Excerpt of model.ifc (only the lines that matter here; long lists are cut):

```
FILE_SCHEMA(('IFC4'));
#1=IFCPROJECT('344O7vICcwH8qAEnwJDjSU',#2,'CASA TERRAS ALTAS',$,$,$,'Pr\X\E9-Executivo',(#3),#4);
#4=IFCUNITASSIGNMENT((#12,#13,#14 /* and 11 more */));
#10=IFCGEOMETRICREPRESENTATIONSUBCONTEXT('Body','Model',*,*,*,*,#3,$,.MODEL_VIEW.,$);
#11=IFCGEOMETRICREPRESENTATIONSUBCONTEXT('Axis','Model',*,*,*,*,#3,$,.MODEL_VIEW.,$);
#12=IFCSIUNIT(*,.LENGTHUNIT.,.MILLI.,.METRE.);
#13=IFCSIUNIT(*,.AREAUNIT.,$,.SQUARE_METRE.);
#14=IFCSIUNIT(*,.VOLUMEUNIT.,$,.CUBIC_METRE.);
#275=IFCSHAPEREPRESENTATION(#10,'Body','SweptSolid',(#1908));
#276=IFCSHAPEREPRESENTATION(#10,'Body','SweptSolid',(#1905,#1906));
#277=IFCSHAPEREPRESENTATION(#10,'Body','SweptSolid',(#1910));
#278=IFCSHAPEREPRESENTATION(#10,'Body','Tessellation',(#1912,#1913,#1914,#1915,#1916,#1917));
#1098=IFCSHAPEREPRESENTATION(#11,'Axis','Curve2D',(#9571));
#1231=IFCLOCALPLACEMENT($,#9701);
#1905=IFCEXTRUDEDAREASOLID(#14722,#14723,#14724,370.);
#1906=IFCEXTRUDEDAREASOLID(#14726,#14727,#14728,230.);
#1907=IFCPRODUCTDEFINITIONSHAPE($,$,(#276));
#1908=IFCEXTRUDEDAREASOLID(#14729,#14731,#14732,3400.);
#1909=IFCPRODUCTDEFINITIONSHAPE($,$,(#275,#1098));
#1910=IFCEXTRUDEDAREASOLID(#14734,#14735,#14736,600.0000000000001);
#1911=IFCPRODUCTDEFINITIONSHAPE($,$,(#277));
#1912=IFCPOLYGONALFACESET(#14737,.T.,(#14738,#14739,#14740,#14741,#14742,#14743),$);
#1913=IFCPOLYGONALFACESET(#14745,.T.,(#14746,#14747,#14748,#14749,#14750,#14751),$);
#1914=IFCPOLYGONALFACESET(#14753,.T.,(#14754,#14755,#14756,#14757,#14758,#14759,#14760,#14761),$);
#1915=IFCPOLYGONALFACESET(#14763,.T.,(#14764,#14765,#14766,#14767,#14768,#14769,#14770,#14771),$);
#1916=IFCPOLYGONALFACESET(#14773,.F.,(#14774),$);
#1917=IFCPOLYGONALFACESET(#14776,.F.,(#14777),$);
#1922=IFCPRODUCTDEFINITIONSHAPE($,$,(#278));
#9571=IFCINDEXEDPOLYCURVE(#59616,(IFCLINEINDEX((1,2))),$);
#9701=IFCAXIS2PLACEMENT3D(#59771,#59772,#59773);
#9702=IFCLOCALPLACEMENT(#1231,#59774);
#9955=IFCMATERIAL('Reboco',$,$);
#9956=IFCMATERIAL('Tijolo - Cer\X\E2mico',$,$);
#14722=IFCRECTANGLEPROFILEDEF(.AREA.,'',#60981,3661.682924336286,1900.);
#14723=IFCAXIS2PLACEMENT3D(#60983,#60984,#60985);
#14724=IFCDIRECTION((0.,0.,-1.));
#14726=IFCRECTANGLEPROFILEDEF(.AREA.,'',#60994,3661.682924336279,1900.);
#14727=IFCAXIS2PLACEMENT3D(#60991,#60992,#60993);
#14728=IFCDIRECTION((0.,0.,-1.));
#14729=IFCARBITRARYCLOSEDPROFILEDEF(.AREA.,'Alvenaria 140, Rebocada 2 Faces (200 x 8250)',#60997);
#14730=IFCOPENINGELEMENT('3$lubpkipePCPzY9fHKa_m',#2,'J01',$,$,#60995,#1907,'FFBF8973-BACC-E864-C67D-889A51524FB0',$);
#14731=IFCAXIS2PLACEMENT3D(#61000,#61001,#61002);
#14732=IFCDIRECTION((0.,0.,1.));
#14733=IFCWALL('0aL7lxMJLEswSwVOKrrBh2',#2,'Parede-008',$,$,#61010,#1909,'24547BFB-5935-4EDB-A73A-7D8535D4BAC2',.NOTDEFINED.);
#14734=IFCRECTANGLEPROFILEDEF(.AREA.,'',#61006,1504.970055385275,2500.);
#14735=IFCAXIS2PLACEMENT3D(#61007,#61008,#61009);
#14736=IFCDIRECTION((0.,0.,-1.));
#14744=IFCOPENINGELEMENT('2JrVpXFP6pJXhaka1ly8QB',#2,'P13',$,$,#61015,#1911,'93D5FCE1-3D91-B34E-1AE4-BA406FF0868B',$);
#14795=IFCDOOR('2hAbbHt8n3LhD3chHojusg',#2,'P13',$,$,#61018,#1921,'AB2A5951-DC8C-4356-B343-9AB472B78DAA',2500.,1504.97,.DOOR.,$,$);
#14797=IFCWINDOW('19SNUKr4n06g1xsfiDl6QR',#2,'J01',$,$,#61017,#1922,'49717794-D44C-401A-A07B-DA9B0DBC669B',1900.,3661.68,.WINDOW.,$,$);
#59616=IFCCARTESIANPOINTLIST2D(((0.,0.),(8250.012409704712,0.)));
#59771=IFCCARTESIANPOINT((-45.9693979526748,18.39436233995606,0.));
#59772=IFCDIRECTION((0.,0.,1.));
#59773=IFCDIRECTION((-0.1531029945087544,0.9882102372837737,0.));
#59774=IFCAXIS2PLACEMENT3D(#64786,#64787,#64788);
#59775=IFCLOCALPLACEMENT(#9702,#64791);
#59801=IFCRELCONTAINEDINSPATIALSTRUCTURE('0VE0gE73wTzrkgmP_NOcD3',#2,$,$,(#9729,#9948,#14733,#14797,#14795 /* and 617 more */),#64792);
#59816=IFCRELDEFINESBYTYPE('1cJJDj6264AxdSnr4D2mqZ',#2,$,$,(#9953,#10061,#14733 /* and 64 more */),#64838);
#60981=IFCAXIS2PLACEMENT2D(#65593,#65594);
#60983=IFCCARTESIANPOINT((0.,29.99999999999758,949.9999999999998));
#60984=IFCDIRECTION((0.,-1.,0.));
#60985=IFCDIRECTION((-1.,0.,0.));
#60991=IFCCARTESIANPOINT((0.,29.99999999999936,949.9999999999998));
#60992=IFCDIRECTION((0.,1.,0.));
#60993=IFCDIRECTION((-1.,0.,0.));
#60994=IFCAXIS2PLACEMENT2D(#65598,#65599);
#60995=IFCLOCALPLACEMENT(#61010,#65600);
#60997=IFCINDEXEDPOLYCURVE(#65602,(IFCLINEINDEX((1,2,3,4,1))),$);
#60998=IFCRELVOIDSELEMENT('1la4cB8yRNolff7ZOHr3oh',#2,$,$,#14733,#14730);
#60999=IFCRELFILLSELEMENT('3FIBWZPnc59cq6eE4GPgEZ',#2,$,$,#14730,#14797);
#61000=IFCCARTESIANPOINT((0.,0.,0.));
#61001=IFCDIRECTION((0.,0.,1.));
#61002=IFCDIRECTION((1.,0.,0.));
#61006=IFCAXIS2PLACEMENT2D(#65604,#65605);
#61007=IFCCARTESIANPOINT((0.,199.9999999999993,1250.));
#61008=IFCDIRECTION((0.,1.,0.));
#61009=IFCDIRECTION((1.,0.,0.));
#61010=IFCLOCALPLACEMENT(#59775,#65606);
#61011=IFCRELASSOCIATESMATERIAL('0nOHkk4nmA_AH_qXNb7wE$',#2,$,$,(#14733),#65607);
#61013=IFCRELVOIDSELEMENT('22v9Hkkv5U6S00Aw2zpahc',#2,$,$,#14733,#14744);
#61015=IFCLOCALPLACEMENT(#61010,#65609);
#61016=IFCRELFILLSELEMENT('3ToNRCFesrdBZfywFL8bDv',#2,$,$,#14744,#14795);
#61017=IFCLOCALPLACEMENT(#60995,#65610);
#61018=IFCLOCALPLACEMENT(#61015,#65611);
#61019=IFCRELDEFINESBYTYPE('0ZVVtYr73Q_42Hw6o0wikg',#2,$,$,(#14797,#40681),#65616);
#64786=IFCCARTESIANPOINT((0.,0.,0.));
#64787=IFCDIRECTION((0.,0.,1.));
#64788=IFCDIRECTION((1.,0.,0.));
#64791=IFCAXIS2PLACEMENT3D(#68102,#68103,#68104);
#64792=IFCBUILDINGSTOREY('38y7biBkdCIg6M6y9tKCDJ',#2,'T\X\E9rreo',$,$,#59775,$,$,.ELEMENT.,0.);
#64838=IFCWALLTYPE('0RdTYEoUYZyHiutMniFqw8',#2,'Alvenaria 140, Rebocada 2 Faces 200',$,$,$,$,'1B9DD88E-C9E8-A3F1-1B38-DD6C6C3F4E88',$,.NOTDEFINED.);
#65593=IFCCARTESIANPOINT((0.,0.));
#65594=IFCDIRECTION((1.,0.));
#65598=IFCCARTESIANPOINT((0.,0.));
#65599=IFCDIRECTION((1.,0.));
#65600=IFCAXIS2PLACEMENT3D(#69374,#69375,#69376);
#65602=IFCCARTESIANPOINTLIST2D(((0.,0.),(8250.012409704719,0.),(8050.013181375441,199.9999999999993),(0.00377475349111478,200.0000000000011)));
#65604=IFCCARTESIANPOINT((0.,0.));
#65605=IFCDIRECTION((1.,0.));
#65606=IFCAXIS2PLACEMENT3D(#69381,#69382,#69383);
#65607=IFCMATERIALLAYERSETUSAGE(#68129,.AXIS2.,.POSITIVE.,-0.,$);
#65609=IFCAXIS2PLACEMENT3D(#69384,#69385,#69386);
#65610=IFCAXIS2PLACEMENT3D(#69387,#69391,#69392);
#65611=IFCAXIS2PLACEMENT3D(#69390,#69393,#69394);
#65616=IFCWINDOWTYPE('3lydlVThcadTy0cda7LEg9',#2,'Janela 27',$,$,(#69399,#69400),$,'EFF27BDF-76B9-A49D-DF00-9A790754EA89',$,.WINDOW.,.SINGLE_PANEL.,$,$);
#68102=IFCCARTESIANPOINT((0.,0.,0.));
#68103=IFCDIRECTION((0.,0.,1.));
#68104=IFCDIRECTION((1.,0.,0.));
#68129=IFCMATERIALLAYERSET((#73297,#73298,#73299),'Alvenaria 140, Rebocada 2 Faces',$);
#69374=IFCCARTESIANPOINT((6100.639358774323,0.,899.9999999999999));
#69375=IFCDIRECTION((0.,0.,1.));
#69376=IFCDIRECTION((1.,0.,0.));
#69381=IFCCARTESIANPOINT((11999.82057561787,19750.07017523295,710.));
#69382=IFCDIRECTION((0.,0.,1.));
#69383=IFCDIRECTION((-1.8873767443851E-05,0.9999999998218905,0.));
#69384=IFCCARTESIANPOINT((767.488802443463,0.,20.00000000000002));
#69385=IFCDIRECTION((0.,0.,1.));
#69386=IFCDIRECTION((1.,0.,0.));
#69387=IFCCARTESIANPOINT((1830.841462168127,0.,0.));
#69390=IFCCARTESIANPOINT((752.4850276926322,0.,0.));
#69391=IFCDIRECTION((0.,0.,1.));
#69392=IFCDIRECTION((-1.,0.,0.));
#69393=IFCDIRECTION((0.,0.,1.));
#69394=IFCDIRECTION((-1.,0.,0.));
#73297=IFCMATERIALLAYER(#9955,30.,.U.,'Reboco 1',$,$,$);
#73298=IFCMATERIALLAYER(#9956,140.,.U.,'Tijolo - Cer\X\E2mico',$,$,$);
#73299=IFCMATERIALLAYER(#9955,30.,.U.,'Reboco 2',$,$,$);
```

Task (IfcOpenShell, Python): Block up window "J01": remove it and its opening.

```python
import ifcopenshell
import ifcopenshell.api.feature
import ifcopenshell.api.root
import ifcopenshell.geom
import ifcopenshell.util.shape

model = ifcopenshell.open("model.ifc")
settings = ifcopenshell.geom.settings()


def volume(element):
    """Net volume in cubic metres, openings subtracted."""
    shape = ifcopenshell.geom.create_shape(settings, element)
    return ifcopenshell.util.shape.get_volume(shape.geometry)


window = model.by_guid("19SNUKr4n06g1xsfiDl6QR")
opening = window.FillsVoids[0].RelatingOpeningElement
wall = opening.VoidsElements[0].RelatingBuildingElement
before = volume(wall)

ifcopenshell.api.root.remove_product(model, product=window)
ifcopenshell.api.feature.remove_feature(model, feature=opening)

after = volume(wall)

print(f"wall volume {before:.3f} -> {after:.3f} m3")

model.write("model-out.ifc")
```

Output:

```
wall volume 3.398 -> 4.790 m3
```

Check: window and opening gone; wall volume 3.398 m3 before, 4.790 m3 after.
